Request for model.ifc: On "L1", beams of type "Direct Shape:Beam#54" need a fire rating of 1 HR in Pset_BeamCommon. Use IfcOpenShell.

First a look at what the model holds.

```python
import ifcopenshell
import ifcopenshell.util.element

model = ifcopenshell.open("model.ifc")
print(model.schema)
storey = next(s for s in model.by_type("IfcBuildingStorey") if s.Name == "L1")
beams = [e for e in ifcopenshell.util.element.get_decomposition(storey) if e.is_a("IfcBeam")]
seen = {}
for e in beams:
    element_type = ifcopenshell.util.element.get_type(e)
    key = (element_type.Name if element_type != e and element_type else None, ifcopenshell.util.element.get_pset(e, "Pset_BeamCommon", "FireRating"))
    seen[key] = seen.get(key, 0) + 1
for (name, value), count in sorted(seen.items(), key=str):
    print(count, "x", name, "|", value)
```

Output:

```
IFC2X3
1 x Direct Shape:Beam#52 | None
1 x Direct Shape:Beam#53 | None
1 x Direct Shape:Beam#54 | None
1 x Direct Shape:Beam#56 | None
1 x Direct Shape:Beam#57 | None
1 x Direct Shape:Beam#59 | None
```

```python
import ifcopenshell
import ifcopenshell.api.pset
import ifcopenshell.util.element

model = ifcopenshell.open("model.ifc")

storey = next(s for s in model.by_type("IfcBuildingStorey") if s.Name == "L1")
beams = [e for e in ifcopenshell.util.element.get_decomposition(storey) if e.is_a("IfcBeam")]

count = 0
for e in beams:
    element_type = ifcopenshell.util.element.get_type(e)
    if element_type in (None, e) or element_type.Name != "Direct Shape:Beam#54":
        continue
    # add_pset returns the element's existing set when there is one.
    pset = ifcopenshell.api.pset.add_pset(model, product=e, name="Pset_BeamCommon")
    ifcopenshell.api.pset.edit_pset(model, pset=pset, properties={"FireRating": "1 HR"})
    count += 1

print(count, "beams updated")

model.write("model_edited.ifc")
```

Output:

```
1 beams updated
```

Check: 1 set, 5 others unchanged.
